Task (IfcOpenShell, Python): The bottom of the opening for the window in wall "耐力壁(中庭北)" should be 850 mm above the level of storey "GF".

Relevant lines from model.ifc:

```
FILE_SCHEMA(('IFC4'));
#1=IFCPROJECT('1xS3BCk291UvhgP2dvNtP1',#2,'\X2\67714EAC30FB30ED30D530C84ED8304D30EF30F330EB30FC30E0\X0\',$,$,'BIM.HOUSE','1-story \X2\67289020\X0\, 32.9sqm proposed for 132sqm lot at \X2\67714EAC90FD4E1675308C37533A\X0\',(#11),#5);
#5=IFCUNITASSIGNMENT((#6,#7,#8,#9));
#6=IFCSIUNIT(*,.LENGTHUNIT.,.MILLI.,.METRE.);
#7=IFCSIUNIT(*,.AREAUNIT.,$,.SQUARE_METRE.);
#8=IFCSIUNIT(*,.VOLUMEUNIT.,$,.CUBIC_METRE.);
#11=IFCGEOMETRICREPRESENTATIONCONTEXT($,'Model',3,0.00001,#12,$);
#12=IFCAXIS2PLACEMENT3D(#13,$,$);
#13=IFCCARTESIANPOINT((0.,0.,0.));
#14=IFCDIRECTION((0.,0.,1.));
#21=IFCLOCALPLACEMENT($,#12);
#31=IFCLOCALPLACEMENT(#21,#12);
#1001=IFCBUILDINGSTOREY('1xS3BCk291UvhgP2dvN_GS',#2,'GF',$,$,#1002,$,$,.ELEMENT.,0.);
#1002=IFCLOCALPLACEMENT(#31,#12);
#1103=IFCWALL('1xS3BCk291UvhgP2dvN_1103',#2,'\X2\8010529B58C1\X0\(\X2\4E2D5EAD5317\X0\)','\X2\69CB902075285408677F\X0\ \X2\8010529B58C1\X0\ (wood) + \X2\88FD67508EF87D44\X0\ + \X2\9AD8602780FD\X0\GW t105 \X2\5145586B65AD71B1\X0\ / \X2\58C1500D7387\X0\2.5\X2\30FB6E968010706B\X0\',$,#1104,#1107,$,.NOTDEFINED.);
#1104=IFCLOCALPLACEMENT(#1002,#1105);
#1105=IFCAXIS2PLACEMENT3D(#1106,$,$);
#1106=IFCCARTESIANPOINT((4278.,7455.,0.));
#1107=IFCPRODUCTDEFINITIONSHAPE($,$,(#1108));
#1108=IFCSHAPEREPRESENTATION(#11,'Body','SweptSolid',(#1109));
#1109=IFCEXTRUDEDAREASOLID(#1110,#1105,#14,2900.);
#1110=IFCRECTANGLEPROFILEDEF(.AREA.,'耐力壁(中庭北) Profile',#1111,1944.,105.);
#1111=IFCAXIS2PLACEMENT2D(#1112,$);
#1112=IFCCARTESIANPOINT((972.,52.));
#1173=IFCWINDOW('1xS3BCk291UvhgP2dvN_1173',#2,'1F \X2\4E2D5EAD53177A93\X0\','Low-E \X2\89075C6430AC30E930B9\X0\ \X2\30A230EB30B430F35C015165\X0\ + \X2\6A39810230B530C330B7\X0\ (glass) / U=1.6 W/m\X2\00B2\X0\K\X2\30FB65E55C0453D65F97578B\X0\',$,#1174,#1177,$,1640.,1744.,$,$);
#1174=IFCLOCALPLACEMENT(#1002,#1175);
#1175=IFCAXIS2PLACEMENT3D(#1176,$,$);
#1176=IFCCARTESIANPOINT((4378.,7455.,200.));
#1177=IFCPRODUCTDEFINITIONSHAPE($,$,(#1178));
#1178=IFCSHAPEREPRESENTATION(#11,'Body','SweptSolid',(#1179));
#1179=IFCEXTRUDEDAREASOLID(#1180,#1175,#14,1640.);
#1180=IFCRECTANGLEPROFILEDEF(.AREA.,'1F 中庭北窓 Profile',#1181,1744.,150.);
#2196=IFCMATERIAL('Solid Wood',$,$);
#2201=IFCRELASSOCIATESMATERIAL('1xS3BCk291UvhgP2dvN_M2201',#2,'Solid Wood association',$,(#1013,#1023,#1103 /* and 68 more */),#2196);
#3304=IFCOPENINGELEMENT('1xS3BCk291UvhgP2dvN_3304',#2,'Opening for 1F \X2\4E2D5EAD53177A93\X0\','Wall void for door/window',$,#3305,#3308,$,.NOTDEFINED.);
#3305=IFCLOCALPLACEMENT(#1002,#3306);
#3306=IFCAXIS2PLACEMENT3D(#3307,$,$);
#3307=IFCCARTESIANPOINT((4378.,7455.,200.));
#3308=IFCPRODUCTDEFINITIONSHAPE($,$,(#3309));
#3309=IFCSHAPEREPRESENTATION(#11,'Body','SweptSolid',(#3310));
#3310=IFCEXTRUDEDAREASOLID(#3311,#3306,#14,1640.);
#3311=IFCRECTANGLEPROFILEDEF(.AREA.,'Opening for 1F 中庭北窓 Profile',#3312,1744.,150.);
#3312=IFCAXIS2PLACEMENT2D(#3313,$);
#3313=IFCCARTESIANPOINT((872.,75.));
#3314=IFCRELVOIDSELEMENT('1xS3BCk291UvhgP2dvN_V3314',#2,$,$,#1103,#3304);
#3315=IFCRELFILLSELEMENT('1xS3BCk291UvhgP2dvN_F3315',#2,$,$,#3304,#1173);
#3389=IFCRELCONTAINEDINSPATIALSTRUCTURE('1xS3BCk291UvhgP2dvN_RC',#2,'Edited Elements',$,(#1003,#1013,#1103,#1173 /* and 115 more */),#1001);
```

```python
import numpy as np
import ifcopenshell
import ifcopenshell.api.geometry
import ifcopenshell.geom
import ifcopenshell.util.element
import ifcopenshell.util.placement
import ifcopenshell.util.shape
import ifcopenshell.util.unit

model = ifcopenshell.open("model.ifc")
unit_scale = ifcopenshell.util.unit.calculate_unit_scale(model)

window = model.by_id(1173)
opening = window.FillsVoids[0].RelatingOpeningElement
storey = ifcopenshell.util.element.get_container(window, ifc_class="IfcBuildingStorey")
level = ifcopenshell.util.placement.get_local_placement(storey.ObjectPlacement)[2, 3]

# The opening's origin need not be at the sill, so measure its lowest point.
shape = ifcopenshell.geom.create_shape(ifcopenshell.geom.settings(), opening)
bottom = ifcopenshell.util.shape.get_shape_bottom_elevation(shape, shape.geometry) / unit_scale
dz = level + 850.0 - bottom

shift = np.array([0.0, 0.0, dz])
# The window is not placed relative to its opening, so move both.
for product in (opening, window):
    matrix = ifcopenshell.util.placement.get_local_placement(product.ObjectPlacement)
    matrix[:3, 3] += shift
    ifcopenshell.api.geometry.edit_object_placement(model, product=product, matrix=matrix, is_si=False)

print(f"moved by {dz * unit_scale:+.3f} m")

model.write("model_edited.ifc")
```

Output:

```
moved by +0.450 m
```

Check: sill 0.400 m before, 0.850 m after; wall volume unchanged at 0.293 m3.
